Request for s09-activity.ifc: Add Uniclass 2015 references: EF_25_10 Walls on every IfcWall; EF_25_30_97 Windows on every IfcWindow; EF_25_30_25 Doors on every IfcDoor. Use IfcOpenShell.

First a look at what the model holds.

```python
import ifcopenshell

model = ifcopenshell.open("s09-activity.ifc")
print(model.schema)
print("classifications:", [c.Name for c in model.by_type("IfcClassification")])
for ifc_class in ("IfcDoor", "IfcRoof", "IfcStair", "IfcWall", "IfcWindow"):
    print(ifc_class, len(model.by_type(ifc_class)))
```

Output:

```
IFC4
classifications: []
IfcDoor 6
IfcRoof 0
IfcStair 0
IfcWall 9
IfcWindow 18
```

```python
import ifcopenshell
import ifcopenshell.api.classification

model = ifcopenshell.open("s09-activity.ifc")

system = ifcopenshell.api.classification.add_classification(model, classification="Uniclass 2015")

codes = {
    "IfcWall": ("EF_25_10", "Walls"),
    "IfcWindow": ("EF_25_30_97", "Windows"),
    "IfcDoor": ("EF_25_30_25", "Doors"),
}
for ifc_class, (code, name) in codes.items():
    products = model.by_type(ifc_class)
    ifcopenshell.api.classification.add_reference(
        model, products=products, classification=system, identification=code, name=name
    )
    print(code, len(products))

model.write("s09-activity_updated.ifc")
```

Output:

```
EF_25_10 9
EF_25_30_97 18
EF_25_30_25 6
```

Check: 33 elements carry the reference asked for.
